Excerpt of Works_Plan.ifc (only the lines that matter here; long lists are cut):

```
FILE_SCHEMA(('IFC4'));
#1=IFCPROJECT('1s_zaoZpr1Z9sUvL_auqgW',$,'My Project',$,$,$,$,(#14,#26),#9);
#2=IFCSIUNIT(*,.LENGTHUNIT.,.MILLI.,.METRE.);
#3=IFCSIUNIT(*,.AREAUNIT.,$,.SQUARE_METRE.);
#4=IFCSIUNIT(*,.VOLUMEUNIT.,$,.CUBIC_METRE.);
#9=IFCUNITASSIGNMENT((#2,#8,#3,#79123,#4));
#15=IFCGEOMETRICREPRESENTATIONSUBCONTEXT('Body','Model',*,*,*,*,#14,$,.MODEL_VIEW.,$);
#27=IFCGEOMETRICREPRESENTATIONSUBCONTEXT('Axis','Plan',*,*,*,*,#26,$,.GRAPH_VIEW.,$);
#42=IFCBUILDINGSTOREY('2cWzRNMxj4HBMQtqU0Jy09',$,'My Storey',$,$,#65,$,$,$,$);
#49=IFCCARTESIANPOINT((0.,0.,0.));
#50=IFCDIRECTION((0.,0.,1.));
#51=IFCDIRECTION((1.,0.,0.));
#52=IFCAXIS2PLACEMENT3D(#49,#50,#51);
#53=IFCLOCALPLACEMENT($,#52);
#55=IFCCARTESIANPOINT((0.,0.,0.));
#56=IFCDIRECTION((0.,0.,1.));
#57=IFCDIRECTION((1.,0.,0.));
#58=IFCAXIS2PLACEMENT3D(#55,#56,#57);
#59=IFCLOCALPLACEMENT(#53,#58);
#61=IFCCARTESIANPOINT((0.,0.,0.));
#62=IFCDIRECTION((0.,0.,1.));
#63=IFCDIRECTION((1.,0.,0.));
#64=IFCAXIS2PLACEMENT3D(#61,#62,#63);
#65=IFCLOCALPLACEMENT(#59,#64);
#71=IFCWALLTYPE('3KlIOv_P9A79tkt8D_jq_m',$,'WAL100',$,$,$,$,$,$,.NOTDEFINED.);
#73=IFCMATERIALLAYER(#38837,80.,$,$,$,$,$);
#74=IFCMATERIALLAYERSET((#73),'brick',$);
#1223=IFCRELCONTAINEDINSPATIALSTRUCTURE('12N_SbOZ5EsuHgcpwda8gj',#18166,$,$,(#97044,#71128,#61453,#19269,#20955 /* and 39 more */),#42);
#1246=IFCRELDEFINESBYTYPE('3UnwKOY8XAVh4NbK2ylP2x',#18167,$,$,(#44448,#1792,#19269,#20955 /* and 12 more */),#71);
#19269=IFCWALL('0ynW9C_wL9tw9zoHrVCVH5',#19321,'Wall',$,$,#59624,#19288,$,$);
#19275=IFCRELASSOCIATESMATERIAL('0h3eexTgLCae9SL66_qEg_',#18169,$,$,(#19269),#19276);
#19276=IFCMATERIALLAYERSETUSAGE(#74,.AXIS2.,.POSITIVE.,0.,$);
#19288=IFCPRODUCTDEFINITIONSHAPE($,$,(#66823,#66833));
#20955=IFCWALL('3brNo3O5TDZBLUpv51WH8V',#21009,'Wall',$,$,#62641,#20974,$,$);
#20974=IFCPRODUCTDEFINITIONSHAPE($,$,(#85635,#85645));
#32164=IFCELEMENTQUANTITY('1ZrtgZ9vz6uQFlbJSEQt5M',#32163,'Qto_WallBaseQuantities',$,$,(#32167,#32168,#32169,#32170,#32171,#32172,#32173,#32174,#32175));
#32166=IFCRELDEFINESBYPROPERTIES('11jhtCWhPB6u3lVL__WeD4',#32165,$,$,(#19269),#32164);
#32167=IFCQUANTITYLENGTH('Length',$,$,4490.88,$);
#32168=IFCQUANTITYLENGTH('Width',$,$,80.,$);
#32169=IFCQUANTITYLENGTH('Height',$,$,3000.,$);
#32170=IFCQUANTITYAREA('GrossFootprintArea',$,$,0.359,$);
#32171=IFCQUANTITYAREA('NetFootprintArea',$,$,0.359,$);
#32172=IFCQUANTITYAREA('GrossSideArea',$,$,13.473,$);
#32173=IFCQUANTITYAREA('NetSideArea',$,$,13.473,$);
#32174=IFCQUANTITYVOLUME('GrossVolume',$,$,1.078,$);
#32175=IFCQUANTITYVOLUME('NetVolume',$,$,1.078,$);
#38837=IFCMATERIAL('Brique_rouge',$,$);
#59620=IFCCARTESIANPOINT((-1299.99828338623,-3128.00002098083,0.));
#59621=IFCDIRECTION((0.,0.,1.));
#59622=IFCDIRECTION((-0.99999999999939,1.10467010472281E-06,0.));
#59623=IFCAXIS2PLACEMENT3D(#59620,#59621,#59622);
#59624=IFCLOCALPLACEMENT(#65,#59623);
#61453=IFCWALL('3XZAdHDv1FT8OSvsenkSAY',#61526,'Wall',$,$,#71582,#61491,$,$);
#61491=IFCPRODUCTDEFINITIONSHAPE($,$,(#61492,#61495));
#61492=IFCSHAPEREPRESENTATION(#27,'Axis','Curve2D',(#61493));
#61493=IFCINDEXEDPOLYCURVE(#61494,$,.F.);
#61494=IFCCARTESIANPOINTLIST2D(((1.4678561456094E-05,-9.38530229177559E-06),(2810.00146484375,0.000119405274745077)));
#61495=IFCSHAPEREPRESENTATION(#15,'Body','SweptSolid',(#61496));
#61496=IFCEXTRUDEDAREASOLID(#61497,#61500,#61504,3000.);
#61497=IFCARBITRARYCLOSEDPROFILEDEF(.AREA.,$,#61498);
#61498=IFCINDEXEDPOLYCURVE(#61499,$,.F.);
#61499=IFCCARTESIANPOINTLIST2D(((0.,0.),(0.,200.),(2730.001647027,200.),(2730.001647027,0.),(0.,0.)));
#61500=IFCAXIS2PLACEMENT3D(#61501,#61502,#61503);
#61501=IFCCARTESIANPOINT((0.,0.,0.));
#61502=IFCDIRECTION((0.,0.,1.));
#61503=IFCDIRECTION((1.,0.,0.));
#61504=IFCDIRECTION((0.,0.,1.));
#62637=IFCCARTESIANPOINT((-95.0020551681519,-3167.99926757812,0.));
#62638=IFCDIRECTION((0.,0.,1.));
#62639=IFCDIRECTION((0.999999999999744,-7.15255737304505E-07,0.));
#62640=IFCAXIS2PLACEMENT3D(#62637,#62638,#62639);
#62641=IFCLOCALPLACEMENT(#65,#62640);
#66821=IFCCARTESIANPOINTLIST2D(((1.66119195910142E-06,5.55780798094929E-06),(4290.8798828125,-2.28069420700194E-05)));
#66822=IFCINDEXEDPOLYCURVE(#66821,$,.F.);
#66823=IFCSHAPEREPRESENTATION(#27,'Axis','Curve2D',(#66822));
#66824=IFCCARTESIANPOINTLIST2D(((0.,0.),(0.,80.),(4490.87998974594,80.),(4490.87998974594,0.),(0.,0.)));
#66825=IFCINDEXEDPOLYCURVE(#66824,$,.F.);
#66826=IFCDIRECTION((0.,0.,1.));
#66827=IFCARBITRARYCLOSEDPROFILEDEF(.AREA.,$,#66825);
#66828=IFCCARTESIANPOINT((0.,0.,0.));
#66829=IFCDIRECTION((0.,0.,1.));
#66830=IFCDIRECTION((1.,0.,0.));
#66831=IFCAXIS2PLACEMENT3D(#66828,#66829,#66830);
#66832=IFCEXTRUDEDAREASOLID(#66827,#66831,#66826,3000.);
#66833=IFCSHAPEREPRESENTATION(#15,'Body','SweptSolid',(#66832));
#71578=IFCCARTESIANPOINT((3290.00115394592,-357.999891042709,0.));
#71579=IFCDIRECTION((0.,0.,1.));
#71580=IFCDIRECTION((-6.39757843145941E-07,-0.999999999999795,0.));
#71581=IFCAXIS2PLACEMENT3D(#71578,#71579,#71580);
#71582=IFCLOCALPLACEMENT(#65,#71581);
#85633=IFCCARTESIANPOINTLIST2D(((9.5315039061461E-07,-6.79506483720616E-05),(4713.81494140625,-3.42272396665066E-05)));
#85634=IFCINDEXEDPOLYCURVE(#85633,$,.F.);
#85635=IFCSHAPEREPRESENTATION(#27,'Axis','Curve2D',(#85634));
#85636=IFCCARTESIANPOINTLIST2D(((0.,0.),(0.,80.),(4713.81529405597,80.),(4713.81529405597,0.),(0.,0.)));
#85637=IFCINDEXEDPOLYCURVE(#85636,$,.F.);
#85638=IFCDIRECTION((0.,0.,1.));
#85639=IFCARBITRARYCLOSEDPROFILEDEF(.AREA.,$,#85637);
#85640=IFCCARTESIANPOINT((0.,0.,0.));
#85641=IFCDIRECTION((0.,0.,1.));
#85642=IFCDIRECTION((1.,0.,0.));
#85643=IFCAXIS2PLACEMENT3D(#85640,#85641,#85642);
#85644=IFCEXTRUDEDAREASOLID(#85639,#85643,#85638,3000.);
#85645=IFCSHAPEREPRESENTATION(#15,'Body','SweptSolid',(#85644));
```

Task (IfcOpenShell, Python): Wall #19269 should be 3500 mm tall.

```python
import ifcopenshell
import ifcopenshell.api.pset
import ifcopenshell.geom
import ifcopenshell.util.element
import ifcopenshell.util.representation
import ifcopenshell.util.shape
import ifcopenshell.util.unit

model = ifcopenshell.open("Works_Plan.ifc")
unit_scale = ifcopenshell.util.unit.calculate_unit_scale(model)
area_scale = ifcopenshell.util.unit.calculate_unit_scale(model, "AREAUNIT")
volume_scale = ifcopenshell.util.unit.calculate_unit_scale(model, "VOLUMEUNIT")
settings = ifcopenshell.geom.settings()


def volume(element):
    """Net volume in cubic metres, openings subtracted."""
    shape = ifcopenshell.geom.create_shape(settings, element)
    return ifcopenshell.util.shape.get_volume(shape.geometry)


wall = model.by_id(19269)
before = volume(wall)

body = ifcopenshell.util.representation.get_representation(wall, "Model", "Body")
solid = body.Items[0]
old_height = solid.Depth
solid.Depth = 3500.0
after = volume(wall)
thickness = 0.08  # wall thickness in metres

# Update the stored height, areas and volumes.
qto = model.by_id(ifcopenshell.util.element.get_pset(wall, "Qto_WallBaseQuantities", should_inherit=False)["id"])
ifcopenshell.api.pset.edit_qto(model, qto=qto, properties={
    "Height": solid.Depth,
    "GrossSideArea": ifcopenshell.util.element.get_pset(wall, "Qto_WallBaseQuantities", "GrossSideArea") * solid.Depth / old_height,
    "NetSideArea": after / thickness / area_scale,
    "GrossVolume": ifcopenshell.util.element.get_pset(wall, "Qto_WallBaseQuantities", "GrossVolume") * solid.Depth / old_height,
    "NetVolume": after / volume_scale,
})

print(f"height {old_height:g} -> {solid.Depth:g}, volume {before:.3f} -> {after:.3f} m3")

model.write("Works_Plan_v2.ifc")
```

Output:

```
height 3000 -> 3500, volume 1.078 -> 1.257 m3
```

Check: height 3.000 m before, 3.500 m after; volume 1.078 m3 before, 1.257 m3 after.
